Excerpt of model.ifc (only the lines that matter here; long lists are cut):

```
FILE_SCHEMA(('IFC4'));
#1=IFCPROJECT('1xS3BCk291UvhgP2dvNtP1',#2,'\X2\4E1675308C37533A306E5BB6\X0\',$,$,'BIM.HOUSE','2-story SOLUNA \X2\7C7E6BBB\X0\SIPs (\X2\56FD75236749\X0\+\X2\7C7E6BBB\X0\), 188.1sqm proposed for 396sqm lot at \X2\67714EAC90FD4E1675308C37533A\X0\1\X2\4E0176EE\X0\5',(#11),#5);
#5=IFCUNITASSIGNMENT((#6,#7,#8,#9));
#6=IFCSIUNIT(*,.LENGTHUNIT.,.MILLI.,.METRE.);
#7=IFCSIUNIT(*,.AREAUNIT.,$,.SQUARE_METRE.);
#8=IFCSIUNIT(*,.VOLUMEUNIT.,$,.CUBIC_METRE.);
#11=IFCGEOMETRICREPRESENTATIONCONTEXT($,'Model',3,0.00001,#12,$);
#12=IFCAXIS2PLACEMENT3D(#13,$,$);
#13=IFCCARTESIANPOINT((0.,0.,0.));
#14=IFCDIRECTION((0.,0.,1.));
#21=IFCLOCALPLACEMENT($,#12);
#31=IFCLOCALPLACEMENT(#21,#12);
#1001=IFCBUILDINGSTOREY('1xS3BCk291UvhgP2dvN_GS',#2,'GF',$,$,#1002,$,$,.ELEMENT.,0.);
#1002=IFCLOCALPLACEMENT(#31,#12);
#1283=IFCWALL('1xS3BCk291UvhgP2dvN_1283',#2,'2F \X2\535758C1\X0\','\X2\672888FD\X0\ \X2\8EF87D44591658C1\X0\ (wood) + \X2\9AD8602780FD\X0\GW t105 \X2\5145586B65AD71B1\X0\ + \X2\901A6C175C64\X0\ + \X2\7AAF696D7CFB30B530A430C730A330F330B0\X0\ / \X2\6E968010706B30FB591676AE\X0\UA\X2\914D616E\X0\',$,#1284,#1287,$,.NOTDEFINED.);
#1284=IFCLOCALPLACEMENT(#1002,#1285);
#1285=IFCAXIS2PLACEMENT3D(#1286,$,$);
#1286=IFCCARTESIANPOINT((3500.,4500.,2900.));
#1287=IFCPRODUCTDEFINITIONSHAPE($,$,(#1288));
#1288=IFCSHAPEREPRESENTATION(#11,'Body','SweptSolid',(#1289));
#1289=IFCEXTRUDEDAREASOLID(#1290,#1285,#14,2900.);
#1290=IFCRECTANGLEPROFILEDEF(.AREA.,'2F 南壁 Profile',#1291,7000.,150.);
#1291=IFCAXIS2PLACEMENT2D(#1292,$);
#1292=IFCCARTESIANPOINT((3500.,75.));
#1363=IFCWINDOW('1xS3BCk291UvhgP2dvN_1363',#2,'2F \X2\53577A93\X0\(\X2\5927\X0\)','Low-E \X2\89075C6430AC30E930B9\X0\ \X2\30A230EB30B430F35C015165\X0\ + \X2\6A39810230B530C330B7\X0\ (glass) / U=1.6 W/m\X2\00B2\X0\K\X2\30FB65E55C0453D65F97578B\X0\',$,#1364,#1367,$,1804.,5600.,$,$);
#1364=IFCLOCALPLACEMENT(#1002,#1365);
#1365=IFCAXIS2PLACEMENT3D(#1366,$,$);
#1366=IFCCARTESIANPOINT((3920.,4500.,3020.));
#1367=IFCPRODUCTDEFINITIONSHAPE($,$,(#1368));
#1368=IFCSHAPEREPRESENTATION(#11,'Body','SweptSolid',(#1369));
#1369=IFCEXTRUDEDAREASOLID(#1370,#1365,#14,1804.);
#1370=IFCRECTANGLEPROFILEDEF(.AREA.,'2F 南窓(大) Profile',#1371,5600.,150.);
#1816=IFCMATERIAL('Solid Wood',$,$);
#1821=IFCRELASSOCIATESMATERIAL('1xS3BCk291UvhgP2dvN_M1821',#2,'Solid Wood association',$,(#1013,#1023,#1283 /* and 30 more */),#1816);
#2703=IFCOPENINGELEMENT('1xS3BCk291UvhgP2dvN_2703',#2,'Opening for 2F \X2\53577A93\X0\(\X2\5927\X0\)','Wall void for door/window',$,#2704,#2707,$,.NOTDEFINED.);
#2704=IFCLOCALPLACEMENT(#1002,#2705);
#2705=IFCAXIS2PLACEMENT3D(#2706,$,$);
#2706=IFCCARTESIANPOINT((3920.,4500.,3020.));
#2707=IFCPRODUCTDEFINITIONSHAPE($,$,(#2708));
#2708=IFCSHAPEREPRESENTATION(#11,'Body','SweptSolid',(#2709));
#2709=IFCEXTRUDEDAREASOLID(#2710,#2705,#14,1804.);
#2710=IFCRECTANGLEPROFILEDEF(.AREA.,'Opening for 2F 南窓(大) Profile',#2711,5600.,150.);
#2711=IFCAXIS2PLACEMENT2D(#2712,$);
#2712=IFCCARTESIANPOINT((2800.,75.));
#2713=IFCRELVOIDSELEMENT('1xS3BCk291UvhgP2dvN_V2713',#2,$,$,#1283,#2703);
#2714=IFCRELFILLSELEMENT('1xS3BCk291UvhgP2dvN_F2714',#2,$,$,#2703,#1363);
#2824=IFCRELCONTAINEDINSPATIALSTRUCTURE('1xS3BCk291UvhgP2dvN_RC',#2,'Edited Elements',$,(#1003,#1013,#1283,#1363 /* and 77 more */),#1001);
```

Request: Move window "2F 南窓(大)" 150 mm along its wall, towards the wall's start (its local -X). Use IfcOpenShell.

```python
import ifcopenshell
import ifcopenshell.api.geometry
import ifcopenshell.util.placement
import ifcopenshell.util.unit

model = ifcopenshell.open("model.ifc")
unit_scale = ifcopenshell.util.unit.calculate_unit_scale(model)

window = model.by_guid("1xS3BCk291UvhgP2dvN_1363")
opening = window.FillsVoids[0].RelatingOpeningElement
wall = opening.VoidsElements[0].RelatingBuildingElement

wall_matrix = ifcopenshell.util.placement.get_local_placement(wall.ObjectPlacement)
shift = wall_matrix[:3, 0] * -0.15 / unit_scale
before = ifcopenshell.util.placement.get_local_placement(window.ObjectPlacement)[:3, 3].copy()

# The window is not placed relative to its opening, so move both.
for product in (opening, window):
    matrix = ifcopenshell.util.placement.get_local_placement(product.ObjectPlacement)
    matrix[:3, 3] += shift
    ifcopenshell.api.geometry.edit_object_placement(model, product=product, matrix=matrix, is_si=False)

after = ifcopenshell.util.placement.get_local_placement(window.ObjectPlacement)[:3, 3]
print("window moved by", (after - before).round(3) + 0.0)

model.write("model-out.ifc")
```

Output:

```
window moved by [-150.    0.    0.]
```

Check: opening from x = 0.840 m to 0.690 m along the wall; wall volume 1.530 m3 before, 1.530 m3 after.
